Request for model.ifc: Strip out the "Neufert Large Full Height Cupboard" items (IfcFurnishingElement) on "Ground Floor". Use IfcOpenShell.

First a look at what the model holds.

```python
import ifcopenshell
import ifcopenshell.util.element

model = ifcopenshell.open("model.ifc")
print(model.schema)
storey = next(s for s in model.by_type("IfcBuildingStorey") if s.Name == "Ground Floor")
furniture = [e for e in ifcopenshell.util.element.get_decomposition(storey) if e.is_a("IfcFurnishingElement")]
seen = {}
for e in furniture:
    element_type = ifcopenshell.util.element.get_type(e)
    name = element_type.Name if element_type not in (None, e) else None
    seen[name] = seen.get(name, 0) + 1
for name, count in sorted(seen.items(), key=str):
    print(count, "x", name)
```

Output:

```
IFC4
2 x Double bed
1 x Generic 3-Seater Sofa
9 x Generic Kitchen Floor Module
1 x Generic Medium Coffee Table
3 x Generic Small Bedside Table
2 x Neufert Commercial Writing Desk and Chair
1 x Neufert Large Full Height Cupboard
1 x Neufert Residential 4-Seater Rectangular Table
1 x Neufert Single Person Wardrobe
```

```python
import ifcopenshell
import ifcopenshell.api.root
import ifcopenshell.util.element

model = ifcopenshell.open("model.ifc")

storey = next(s for s in model.by_type("IfcBuildingStorey") if s.Name == "Ground Floor")
furniture = [e for e in ifcopenshell.util.element.get_decomposition(storey) if e.is_a("IfcFurnishingElement")]
targets = [e for e in furniture if (t := ifcopenshell.util.element.get_type(e)) not in (None, e) and t.Name == "Neufert Large Full Height Cupboard"]

for e in targets:
    ifcopenshell.api.root.remove_product(model, product=e)
print(len(targets), "removed")

model.write("model_v2.ifc")
```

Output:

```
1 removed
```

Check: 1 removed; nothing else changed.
